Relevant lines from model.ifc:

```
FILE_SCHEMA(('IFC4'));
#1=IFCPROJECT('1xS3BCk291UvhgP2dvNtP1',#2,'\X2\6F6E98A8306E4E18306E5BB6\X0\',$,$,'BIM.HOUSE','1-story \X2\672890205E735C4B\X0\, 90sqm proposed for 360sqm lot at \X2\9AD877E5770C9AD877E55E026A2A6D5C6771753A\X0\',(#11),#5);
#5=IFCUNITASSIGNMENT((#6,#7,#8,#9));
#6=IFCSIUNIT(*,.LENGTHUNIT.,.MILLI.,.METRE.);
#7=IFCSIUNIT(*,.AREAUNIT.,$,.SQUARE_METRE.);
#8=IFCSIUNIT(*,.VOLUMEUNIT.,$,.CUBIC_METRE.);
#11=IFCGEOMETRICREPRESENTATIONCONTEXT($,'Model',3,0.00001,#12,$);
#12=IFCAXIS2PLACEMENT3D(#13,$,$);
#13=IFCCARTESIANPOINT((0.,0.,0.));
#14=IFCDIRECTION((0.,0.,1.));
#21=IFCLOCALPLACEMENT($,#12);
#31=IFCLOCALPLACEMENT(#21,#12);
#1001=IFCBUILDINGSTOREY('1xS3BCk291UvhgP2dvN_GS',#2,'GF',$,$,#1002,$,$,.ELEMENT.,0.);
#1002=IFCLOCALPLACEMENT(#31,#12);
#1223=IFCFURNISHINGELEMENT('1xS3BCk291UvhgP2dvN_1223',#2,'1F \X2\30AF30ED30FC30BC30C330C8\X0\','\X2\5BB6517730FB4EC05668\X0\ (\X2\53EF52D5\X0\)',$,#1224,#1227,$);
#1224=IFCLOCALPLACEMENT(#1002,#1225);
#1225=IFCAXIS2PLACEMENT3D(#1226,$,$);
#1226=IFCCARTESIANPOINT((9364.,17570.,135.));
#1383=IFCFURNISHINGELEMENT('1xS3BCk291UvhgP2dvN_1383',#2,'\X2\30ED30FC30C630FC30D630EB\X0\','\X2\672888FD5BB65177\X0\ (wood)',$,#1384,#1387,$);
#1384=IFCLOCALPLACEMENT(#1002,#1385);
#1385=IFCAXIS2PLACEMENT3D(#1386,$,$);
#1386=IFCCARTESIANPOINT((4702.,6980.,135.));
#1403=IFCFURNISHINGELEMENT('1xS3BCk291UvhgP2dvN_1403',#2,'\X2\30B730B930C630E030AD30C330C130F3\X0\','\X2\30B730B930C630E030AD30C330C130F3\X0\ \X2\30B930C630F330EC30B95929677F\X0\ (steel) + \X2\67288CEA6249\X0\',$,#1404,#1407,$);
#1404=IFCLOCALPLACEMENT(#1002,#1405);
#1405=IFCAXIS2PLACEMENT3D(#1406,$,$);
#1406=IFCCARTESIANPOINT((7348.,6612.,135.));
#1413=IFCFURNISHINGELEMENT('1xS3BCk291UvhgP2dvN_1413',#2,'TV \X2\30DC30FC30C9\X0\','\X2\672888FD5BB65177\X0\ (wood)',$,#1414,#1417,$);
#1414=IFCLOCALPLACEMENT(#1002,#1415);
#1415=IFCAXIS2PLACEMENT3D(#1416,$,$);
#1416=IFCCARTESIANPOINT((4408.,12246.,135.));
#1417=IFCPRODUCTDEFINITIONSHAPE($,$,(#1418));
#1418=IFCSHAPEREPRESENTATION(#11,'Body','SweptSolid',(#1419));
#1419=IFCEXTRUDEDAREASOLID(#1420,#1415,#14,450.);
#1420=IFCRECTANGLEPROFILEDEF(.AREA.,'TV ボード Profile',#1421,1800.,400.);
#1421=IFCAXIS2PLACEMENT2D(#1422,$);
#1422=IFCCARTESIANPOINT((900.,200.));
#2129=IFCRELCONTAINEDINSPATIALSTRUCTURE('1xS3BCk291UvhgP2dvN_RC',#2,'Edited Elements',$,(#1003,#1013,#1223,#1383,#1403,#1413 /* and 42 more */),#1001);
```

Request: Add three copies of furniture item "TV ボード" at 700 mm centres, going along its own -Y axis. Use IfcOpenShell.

```python
import ifcopenshell
import ifcopenshell.api.geometry
import ifcopenshell.api.root
import ifcopenshell.util.element
import ifcopenshell.util.placement

model = ifcopenshell.open("model.ifc")


def reuse_history(source, copy):
    """copy_class also copies each property set's owner history, people and application; keep the originals."""
    for rel in copy.IsDefinedBy:
        if rel.is_a("IfcRelDefinesByProperties") and (history := rel.RelatingPropertyDefinition.OwnerHistory):
            rel.RelatingPropertyDefinition.OwnerHistory = source.OwnerHistory
            ifcopenshell.util.element.remove_deep2(model, history)


source = model.by_guid("1xS3BCk291UvhgP2dvN_1413")
base = ifcopenshell.util.placement.get_local_placement(source.ObjectPlacement)
step = -base[:3, 1] * 700.0

for i in range(1, 4):
    copy = ifcopenshell.api.root.copy_class(model, product=source)
    copy.Representation = ifcopenshell.util.element.copy_deep(
        model, source.Representation, exclude=["IfcGeometricRepresentationContext", "IfcRepresentationMap"]
    )
    reuse_history(source, copy)
    matrix = base.copy()
    matrix[:3, 3] += i * step
    print("added at", matrix[:3, 3].round(3) + 0.0)
    ifcopenshell.api.geometry.edit_object_placement(model, product=copy, matrix=matrix, is_si=False)

model.write("model_updated.ifc")
```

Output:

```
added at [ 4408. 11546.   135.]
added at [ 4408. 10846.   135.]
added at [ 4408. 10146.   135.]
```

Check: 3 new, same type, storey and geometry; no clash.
